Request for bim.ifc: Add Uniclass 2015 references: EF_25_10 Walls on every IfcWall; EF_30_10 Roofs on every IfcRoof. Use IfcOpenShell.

First a look at what the model holds.

```python
import ifcopenshell

model = ifcopenshell.open("bim.ifc")
print(model.schema)
print("classifications:", [c.Name for c in model.by_type("IfcClassification")])
for ifc_class in ("IfcDoor", "IfcRoof", "IfcStair", "IfcWall", "IfcWindow"):
    print(ifc_class, len(model.by_type(ifc_class)))
```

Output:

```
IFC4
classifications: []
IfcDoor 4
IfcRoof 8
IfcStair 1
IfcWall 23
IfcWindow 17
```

```python
import ifcopenshell
import ifcopenshell.api.classification

model = ifcopenshell.open("bim.ifc")

system = ifcopenshell.api.classification.add_classification(model, classification="Uniclass 2015")

codes = {
    "IfcWall": ("EF_25_10", "Walls"),
    "IfcRoof": ("EF_30_10", "Roofs"),
}
for ifc_class, (code, name) in codes.items():
    products = model.by_type(ifc_class)
    ifcopenshell.api.classification.add_reference(
        model, products=products, classification=system, identification=code, name=name
    )
    print(code, len(products))

model.write("bim_updated.ifc")
```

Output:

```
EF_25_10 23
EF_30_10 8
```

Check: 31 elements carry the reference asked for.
